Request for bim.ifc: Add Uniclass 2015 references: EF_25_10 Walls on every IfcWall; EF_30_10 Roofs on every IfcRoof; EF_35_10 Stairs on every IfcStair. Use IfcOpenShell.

First a look at what the model holds.

```python
import ifcopenshell

model = ifcopenshell.open("bim.ifc")
print(model.schema)
print("classifications:", [c.Name for c in model.by_type("IfcClassification")])
for ifc_class in ("IfcDoor", "IfcRoof", "IfcStair", "IfcWall", "IfcWindow"):
    print(ifc_class, len(model.by_type(ifc_class)))
```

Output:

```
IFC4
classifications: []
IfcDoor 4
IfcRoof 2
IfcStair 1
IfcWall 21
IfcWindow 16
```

```python
import ifcopenshell
import ifcopenshell.api.classification

model = ifcopenshell.open("bim.ifc")

system = ifcopenshell.api.classification.add_classification(model, classification="Uniclass 2015")

codes = {
    "IfcWall": ("EF_25_10", "Walls"),
    "IfcRoof": ("EF_30_10", "Roofs"),
    "IfcStair": ("EF_35_10", "Stairs"),
}
for ifc_class, (code, name) in codes.items():
    products = model.by_type(ifc_class)
    ifcopenshell.api.classification.add_reference(
        model, products=products, classification=system, identification=code, name=name
    )
    print(code, len(products))

model.write("bim_v2.ifc")
```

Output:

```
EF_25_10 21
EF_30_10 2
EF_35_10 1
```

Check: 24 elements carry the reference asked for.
